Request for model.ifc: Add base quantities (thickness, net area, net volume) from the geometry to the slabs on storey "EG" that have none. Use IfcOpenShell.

First a look at what the model holds.

```python
import ifcopenshell
import ifcopenshell.util.element
import ifcopenshell.util.unit

model = ifcopenshell.open("model.ifc")
print(model.schema)
for unit_type in ("LENGTHUNIT", "AREAUNIT", "VOLUMEUNIT"):
    print(unit_type, ifcopenshell.util.unit.calculate_unit_scale(model, unit_type))
storey = next(s for s in model.by_type("IfcBuildingStorey") if s.Name == "EG")
slabs = [e for e in ifcopenshell.util.element.get_decomposition(storey) if e.is_a("IfcSlab")]
for e in sorted(slabs, key=lambda e: e.id()):
    print(e.id(), e.is_a(), e.Name, list(ifcopenshell.util.element.get_psets(e, qtos_only=True)), sep=" | ")
```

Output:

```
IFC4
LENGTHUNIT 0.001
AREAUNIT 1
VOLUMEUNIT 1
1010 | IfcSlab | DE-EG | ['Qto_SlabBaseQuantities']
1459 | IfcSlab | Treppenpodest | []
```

```python
import ifcopenshell
import ifcopenshell.api.pset
import ifcopenshell.geom
import ifcopenshell.util.element
import ifcopenshell.util.shape
import ifcopenshell.util.unit

model = ifcopenshell.open("model.ifc")
unit_scale = ifcopenshell.util.unit.calculate_unit_scale(model)
area_scale = ifcopenshell.util.unit.calculate_unit_scale(model, "AREAUNIT")
volume_scale = ifcopenshell.util.unit.calculate_unit_scale(model, "VOLUMEUNIT")
settings = ifcopenshell.geom.settings()

storey = next(s for s in model.by_type("IfcBuildingStorey") if s.Name == "EG")
slabs = [e for e in ifcopenshell.util.element.get_decomposition(storey) if e.is_a("IfcSlab")]

for e in sorted(slabs, key=lambda e: e.id()):
    if ifcopenshell.util.element.get_psets(e, qtos_only=True, should_inherit=False):
        continue
    # Geometry comes back in metres, in the element's own axes.
    shape = ifcopenshell.geom.create_shape(settings, e)
    values = {
        "Width": ifcopenshell.util.shape.get_z(shape.geometry) / unit_scale,
        "NetArea": ifcopenshell.util.shape.get_footprint_area(shape.geometry) / area_scale,
        "NetVolume": ifcopenshell.util.shape.get_volume(shape.geometry) / volume_scale,
    }
    qto = ifcopenshell.api.pset.add_qto(model, product=e, name="Qto_SlabBaseQuantities")
    ifcopenshell.api.pset.edit_qto(model, qto=qto, properties=values)
    print(e.id(), {k: round(v, 3) for k, v in values.items()})

model.write("model-out.ifc")
```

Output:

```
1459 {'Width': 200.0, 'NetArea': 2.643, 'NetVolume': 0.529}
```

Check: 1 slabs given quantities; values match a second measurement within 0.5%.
